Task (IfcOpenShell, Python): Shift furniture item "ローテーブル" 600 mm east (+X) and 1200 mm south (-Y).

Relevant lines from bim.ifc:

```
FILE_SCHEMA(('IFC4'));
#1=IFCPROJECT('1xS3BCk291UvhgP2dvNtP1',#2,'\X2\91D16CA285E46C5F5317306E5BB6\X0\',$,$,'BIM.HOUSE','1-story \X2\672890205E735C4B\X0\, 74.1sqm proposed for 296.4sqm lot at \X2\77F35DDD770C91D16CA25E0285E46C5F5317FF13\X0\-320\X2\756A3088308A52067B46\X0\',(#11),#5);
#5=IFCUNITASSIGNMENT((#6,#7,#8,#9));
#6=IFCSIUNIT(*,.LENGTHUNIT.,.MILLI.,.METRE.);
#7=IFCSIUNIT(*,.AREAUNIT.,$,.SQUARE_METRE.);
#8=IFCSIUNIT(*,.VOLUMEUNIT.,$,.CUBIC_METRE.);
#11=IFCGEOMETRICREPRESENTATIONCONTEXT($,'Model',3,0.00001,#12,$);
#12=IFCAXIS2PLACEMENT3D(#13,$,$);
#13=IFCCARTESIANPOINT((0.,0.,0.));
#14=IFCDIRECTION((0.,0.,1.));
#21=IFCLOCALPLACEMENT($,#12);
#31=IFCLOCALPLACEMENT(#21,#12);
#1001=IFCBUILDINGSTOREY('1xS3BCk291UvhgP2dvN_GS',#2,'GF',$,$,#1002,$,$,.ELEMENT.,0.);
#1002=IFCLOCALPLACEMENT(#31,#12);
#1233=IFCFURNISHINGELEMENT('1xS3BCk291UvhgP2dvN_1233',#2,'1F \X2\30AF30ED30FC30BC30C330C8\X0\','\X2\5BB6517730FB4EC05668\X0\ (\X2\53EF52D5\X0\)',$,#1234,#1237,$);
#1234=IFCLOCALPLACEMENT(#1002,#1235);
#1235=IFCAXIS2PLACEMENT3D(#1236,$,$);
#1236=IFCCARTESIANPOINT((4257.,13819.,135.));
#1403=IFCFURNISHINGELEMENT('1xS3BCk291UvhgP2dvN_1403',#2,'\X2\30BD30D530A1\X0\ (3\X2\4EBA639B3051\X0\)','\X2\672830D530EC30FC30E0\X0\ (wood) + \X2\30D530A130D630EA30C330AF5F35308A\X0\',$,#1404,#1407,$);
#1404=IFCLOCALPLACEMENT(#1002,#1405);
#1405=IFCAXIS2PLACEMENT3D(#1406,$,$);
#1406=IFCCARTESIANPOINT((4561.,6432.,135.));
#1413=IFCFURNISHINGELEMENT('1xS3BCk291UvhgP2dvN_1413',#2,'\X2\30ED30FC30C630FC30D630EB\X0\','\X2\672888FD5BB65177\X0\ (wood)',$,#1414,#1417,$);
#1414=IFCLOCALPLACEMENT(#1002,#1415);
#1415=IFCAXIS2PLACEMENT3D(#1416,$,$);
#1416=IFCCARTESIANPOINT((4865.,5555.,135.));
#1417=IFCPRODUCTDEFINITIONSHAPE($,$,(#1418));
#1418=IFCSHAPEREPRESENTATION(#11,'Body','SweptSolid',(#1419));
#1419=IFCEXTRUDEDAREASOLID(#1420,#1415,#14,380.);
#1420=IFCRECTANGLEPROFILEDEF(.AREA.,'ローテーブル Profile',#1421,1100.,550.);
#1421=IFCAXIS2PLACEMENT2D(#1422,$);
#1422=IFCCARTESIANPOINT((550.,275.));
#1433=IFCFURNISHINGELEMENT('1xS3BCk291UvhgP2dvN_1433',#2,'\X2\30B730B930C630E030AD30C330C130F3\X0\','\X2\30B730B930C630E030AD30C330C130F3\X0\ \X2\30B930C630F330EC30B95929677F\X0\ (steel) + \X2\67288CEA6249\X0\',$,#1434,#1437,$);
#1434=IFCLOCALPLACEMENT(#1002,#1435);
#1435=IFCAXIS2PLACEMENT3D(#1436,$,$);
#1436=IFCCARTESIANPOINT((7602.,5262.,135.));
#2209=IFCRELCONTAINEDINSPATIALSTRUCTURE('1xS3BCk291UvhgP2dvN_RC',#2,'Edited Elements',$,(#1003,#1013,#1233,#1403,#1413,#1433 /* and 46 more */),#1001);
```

```python
import ifcopenshell
import ifcopenshell.api.geometry
import ifcopenshell.util.placement
import ifcopenshell.util.unit

model = ifcopenshell.open("bim.ifc")
unit_scale = ifcopenshell.util.unit.calculate_unit_scale(model)

item = model.by_guid("1xS3BCk291UvhgP2dvN_1413")
matrix = ifcopenshell.util.placement.get_local_placement(item.ObjectPlacement)
matrix[0, 3] += 0.6 / unit_scale
matrix[1, 3] -= 1.2 / unit_scale
ifcopenshell.api.geometry.edit_object_placement(model, product=item, matrix=matrix, is_si=False)

print(ifcopenshell.util.placement.get_local_placement(item.ObjectPlacement).round(3) + 0.0)

model.write("bim_rev.ifc")
```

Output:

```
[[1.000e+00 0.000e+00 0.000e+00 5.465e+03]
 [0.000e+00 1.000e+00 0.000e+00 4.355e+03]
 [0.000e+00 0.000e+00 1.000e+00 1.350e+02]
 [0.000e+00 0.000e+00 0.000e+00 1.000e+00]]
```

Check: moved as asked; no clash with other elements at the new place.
